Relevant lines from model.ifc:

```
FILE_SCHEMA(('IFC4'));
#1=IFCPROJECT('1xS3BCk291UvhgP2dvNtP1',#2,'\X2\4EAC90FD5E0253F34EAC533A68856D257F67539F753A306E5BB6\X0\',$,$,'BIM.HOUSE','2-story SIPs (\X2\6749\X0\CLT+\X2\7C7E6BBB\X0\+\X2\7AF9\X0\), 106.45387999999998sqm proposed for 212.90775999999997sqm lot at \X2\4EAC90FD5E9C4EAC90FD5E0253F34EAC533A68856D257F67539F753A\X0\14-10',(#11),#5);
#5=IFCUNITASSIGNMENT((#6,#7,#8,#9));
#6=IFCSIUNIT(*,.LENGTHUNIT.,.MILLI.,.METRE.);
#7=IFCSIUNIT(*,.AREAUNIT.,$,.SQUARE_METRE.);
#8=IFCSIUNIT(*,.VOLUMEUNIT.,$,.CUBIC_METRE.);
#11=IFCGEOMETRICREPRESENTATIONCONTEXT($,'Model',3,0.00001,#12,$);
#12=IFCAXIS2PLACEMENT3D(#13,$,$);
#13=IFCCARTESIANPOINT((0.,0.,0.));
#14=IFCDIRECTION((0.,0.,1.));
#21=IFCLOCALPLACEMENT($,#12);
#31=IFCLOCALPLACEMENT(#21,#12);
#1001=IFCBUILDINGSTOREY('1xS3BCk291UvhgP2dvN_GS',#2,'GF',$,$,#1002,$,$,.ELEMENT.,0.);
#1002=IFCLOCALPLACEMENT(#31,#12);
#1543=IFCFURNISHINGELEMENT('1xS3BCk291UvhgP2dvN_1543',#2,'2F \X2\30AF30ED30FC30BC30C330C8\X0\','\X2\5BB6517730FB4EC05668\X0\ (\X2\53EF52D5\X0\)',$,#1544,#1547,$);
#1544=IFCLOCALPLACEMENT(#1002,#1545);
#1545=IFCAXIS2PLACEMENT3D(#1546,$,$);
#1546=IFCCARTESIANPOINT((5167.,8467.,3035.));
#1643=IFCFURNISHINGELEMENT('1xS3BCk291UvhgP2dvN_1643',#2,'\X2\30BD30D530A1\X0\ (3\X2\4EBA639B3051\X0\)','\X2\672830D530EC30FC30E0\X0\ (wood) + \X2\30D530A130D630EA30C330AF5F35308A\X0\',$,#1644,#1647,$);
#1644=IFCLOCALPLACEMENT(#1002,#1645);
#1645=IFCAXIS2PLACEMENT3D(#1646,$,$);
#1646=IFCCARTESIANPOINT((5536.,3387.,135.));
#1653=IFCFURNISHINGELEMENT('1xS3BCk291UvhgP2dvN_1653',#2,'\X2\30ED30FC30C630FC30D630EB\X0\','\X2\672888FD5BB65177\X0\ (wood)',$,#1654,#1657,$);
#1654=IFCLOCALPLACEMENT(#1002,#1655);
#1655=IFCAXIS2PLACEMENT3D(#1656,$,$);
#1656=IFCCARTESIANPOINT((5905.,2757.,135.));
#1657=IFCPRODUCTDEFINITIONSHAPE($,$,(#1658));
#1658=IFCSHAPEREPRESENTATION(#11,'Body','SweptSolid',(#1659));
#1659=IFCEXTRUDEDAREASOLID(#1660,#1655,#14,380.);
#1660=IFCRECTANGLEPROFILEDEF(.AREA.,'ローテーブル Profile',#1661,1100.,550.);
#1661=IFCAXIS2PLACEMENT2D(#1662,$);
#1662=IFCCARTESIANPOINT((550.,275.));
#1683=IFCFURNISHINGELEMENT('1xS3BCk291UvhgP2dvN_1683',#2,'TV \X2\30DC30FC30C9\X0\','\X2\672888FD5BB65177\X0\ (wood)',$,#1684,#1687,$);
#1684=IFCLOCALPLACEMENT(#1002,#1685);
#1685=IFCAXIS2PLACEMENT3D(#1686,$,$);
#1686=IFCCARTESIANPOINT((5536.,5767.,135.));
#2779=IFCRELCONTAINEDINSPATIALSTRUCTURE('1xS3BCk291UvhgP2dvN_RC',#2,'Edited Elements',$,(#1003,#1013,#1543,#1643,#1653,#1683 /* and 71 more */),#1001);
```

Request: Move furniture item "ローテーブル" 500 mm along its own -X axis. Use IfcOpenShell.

```python
import ifcopenshell
import ifcopenshell.api.geometry
import ifcopenshell.util.placement

model = ifcopenshell.open("model.ifc")

item = model.by_guid("1xS3BCk291UvhgP2dvN_1653")
matrix = ifcopenshell.util.placement.get_local_placement(item.ObjectPlacement)
matrix[:3, 3] -= matrix[:3, 0] * 500.0
ifcopenshell.api.geometry.edit_object_placement(model, product=item, matrix=matrix, is_si=False)

print(ifcopenshell.util.placement.get_local_placement(item.ObjectPlacement).round(3) + 0.0)

model.write("model-out.ifc")
```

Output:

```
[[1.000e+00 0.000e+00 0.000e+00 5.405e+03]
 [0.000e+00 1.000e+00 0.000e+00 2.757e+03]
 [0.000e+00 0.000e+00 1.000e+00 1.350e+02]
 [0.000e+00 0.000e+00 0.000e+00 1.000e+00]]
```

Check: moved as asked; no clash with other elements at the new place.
